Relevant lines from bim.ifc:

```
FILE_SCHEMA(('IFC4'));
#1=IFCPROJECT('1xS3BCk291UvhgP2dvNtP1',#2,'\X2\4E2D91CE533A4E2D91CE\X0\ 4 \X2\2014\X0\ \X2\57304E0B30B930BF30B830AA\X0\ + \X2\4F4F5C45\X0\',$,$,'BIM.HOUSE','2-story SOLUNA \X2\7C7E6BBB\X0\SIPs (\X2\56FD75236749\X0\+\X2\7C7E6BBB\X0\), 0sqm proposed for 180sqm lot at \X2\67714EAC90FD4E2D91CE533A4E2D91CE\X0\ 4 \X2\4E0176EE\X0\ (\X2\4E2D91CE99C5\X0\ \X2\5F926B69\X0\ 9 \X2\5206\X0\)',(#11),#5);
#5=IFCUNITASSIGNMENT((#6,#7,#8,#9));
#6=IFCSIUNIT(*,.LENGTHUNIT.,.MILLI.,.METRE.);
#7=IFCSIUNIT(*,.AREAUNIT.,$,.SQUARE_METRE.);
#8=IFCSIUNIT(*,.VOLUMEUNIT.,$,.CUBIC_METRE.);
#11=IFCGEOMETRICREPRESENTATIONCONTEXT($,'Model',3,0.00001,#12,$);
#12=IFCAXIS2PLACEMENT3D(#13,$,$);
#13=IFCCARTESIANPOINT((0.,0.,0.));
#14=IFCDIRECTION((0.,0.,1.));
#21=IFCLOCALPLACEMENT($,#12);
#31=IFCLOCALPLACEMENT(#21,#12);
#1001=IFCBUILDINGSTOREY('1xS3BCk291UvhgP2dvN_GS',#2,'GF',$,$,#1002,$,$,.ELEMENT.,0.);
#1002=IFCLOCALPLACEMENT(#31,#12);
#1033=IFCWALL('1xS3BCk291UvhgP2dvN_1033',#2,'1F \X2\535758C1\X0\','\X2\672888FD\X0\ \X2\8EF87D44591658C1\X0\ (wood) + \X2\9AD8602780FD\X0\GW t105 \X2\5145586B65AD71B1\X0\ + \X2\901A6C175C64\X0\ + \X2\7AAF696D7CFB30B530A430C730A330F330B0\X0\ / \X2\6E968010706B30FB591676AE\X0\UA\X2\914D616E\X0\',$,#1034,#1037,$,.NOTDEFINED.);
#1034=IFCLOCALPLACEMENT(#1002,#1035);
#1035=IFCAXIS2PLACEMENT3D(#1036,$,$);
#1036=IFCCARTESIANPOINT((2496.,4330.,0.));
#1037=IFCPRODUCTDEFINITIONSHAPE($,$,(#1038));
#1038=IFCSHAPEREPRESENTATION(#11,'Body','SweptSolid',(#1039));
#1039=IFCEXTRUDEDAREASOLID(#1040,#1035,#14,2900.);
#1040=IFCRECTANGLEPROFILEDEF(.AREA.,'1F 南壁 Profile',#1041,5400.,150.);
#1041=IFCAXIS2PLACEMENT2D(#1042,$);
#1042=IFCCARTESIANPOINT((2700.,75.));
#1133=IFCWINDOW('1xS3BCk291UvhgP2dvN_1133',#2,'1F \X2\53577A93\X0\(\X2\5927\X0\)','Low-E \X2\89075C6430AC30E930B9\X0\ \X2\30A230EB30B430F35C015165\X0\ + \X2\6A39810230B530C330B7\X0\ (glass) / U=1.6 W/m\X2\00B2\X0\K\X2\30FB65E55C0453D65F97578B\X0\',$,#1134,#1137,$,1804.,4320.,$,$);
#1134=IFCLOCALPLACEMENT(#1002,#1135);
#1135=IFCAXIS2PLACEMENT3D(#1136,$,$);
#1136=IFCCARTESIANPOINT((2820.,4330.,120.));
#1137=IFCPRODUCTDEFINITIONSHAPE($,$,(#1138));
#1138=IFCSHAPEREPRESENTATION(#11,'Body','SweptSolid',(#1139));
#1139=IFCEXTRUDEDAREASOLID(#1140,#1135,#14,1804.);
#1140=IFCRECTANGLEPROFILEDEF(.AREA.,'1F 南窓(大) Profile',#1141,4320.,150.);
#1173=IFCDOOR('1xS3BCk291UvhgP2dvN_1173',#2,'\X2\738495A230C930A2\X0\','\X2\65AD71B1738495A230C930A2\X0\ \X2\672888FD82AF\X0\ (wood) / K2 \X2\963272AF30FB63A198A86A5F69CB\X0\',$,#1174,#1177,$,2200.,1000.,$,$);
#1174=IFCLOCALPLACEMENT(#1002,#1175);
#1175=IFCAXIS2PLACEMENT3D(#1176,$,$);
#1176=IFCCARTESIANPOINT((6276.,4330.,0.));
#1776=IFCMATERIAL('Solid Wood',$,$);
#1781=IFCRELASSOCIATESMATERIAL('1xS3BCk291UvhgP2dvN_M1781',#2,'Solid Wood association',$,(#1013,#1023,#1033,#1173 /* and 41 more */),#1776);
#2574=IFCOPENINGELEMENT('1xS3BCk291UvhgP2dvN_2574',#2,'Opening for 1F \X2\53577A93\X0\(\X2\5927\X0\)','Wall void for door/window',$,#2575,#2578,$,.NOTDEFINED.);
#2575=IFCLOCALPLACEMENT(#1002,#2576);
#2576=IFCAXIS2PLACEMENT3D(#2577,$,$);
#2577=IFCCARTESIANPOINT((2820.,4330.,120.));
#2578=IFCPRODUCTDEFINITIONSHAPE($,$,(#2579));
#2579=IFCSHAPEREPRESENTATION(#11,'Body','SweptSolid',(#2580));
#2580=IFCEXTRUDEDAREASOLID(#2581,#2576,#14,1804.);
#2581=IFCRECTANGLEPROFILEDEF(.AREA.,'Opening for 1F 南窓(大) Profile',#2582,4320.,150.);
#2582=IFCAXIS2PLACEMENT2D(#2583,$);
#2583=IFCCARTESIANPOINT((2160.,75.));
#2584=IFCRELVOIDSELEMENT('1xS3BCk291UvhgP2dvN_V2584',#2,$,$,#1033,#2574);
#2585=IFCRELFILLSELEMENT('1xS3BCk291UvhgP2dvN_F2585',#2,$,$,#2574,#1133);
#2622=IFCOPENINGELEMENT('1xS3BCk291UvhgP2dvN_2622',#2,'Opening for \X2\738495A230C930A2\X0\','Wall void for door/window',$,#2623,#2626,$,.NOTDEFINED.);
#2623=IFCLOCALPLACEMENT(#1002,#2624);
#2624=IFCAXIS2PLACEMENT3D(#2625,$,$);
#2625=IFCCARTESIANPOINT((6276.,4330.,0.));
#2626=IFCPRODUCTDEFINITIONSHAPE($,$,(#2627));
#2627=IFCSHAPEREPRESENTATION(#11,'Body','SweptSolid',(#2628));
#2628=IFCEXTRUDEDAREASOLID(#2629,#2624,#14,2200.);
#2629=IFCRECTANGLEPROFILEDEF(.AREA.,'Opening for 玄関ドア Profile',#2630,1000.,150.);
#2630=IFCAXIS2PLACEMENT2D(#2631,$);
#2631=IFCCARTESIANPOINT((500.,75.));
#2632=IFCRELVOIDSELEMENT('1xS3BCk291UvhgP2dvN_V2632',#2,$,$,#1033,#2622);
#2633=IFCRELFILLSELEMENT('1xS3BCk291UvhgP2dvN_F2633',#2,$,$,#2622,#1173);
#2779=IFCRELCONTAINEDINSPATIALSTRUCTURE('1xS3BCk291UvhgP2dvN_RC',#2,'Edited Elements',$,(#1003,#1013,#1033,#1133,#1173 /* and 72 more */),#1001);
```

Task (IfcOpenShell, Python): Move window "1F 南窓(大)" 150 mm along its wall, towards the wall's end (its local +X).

```python
import ifcopenshell
import ifcopenshell.api.geometry
import ifcopenshell.util.placement
import ifcopenshell.util.unit

model = ifcopenshell.open("bim.ifc")
unit_scale = ifcopenshell.util.unit.calculate_unit_scale(model)

window = model.by_guid("1xS3BCk291UvhgP2dvN_1133")
opening = window.FillsVoids[0].RelatingOpeningElement
wall = opening.VoidsElements[0].RelatingBuildingElement

wall_matrix = ifcopenshell.util.placement.get_local_placement(wall.ObjectPlacement)
shift = wall_matrix[:3, 0] * 0.15 / unit_scale
before = ifcopenshell.util.placement.get_local_placement(window.ObjectPlacement)[:3, 3].copy()

# The window is not placed relative to its opening, so move both.
for product in (opening, window):
    matrix = ifcopenshell.util.placement.get_local_placement(product.ObjectPlacement)
    matrix[:3, 3] += shift
    ifcopenshell.api.geometry.edit_object_placement(model, product=product, matrix=matrix, is_si=False)

after = ifcopenshell.util.placement.get_local_placement(window.ObjectPlacement)[:3, 3]
print("window moved by", (after - before).round(3) + 0.0)

model.write("bim_rev.ifc")
```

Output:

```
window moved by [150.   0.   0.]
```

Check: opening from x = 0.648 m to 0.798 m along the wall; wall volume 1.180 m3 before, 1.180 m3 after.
